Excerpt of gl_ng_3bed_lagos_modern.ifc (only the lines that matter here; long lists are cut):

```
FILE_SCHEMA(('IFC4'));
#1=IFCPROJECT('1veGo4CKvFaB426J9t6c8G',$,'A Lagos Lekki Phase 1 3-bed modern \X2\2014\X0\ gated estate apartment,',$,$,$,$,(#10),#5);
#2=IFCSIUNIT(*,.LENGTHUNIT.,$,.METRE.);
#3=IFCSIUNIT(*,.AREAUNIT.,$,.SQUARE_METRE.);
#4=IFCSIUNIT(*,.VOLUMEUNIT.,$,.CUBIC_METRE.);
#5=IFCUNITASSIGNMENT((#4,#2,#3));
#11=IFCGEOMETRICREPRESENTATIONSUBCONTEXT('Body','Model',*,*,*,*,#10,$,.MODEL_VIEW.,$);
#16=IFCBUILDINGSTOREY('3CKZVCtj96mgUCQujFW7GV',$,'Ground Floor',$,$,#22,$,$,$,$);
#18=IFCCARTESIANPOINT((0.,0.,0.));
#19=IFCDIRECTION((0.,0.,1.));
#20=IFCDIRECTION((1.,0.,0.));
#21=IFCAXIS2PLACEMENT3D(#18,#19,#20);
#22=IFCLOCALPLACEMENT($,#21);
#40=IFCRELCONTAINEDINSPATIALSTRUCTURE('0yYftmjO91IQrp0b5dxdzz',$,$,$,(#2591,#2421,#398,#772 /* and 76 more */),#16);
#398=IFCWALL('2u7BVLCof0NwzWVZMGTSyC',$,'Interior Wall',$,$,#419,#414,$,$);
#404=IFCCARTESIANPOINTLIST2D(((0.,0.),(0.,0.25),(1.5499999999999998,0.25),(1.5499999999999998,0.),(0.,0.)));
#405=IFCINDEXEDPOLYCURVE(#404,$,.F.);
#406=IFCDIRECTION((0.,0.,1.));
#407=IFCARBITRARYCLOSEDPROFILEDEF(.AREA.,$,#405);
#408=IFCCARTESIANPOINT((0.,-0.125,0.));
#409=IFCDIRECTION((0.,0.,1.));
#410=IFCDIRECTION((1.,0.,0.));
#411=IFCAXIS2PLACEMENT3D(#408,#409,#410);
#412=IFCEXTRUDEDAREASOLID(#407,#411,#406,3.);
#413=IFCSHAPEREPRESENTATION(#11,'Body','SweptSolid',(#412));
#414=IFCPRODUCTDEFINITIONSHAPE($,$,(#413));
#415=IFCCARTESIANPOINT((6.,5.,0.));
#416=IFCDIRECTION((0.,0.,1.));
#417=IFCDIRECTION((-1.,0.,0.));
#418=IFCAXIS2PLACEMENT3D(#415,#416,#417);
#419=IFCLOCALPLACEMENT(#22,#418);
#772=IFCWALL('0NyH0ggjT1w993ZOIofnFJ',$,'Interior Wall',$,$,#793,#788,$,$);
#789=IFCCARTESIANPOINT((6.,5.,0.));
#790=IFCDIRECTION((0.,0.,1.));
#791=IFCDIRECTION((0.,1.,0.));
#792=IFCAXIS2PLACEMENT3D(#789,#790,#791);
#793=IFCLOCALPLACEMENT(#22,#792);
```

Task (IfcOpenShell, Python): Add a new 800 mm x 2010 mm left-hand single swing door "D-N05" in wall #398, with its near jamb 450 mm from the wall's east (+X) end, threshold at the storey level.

```python
import numpy as np
import ifcopenshell
import ifcopenshell.api.feature
import ifcopenshell.api.geometry
import ifcopenshell.api.root
import ifcopenshell.api.spatial
import ifcopenshell.geom
import ifcopenshell.util.element
import ifcopenshell.util.placement
import ifcopenshell.util.representation
import ifcopenshell.util.shape
import ifcopenshell.util.unit

model = ifcopenshell.open("gl_ng_3bed_lagos_modern.ifc")
unit_scale = ifcopenshell.util.unit.calculate_unit_scale(model)
settings = ifcopenshell.geom.settings()


def volume(element):
    """Net volume in cubic metres, openings subtracted."""
    shape = ifcopenshell.geom.create_shape(settings, element)
    return ifcopenshell.util.shape.get_volume(shape.geometry)


wall = model.by_guid("2u7BVLCof0NwzWVZMGTSyC")
storey = ifcopenshell.util.element.get_container(wall, ifc_class="IfcBuildingStorey")
context = ifcopenshell.util.representation.get_context(model, "Model", "Body", "MODEL_VIEW")
before = volume(wall)

width, height, from_end, sill = 0.8, 2.01, 0.45, 0.0  # metres

# The wall runs along its own X axis, and the end named is its -X end.
wall_shape = ifcopenshell.geom.create_shape(settings, wall)
x, y, z = ifcopenshell.util.shape.get_vertices(wall_shape.geometry).T
start = x.min() + from_end
face, thickness = float(y.min()), float(y.max() - y.min())
wall_matrix = ifcopenshell.util.placement.get_local_placement(wall.ObjectPlacement)
level = ifcopenshell.util.placement.get_local_placement(storey.ObjectPlacement)[2, 3]


def in_wall(x, y):
    """Placement at x, y metres in the wall's axes, at sill height."""
    matrix = wall_matrix.copy()
    matrix[:, 3] = wall_matrix @ np.array([x / unit_scale, y / unit_scale, 0.0, 1.0])
    matrix[2, 3] = level + sill / unit_scale
    return matrix


# Opening: a box that overshoots both wall faces by 50 mm.
opening = ifcopenshell.api.root.create_entity(model, ifc_class="IfcOpeningElement", predefined_type="OPENING")
box = ifcopenshell.api.geometry.add_wall_representation(
    model, context=context, length=width, height=height, thickness=thickness + 0.1
)
ifcopenshell.api.geometry.assign_representation(model, product=opening, representation=box)
ifcopenshell.api.geometry.edit_object_placement(model, product=opening, matrix=in_wall(start, face - 0.05), is_si=False)
ifcopenshell.api.feature.add_feature(model, feature=opening, element=wall)

door = ifcopenshell.api.root.create_entity(model, ifc_class="IfcDoor", name="D-N05", predefined_type="DOOR")
door.OverallWidth, door.OverallHeight = width / unit_scale, height / unit_scale
door.OperationType = "SINGLE_SWING_LEFT"
body = ifcopenshell.api.geometry.add_door_representation(
    model,
    context=context,
    overall_width=door.OverallWidth,
    overall_height=door.OverallHeight,
    operation_type="SINGLE_SWING_LEFT",
    lining_properties={"LiningDepth": thickness / unit_scale, "ThresholdDepth": thickness / unit_scale},
)
ifcopenshell.api.geometry.assign_representation(model, product=door, representation=body)
ifcopenshell.api.spatial.assign_container(model, products=[door], relating_structure=storey)
ifcopenshell.api.feature.add_filling(model, opening=opening, element=door)

# The lining spans the wall, so the door starts at the wall face.
ifcopenshell.api.geometry.edit_object_placement(model, product=door, matrix=in_wall(start, face), is_si=False)

after = volume(wall)

print(f"wall volume {before:.3f} -> {after:.3f} m3")

model.write("gl_ng_3bed_lagos_modern-out.ifc")
```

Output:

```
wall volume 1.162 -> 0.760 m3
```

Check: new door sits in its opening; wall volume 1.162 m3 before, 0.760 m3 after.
